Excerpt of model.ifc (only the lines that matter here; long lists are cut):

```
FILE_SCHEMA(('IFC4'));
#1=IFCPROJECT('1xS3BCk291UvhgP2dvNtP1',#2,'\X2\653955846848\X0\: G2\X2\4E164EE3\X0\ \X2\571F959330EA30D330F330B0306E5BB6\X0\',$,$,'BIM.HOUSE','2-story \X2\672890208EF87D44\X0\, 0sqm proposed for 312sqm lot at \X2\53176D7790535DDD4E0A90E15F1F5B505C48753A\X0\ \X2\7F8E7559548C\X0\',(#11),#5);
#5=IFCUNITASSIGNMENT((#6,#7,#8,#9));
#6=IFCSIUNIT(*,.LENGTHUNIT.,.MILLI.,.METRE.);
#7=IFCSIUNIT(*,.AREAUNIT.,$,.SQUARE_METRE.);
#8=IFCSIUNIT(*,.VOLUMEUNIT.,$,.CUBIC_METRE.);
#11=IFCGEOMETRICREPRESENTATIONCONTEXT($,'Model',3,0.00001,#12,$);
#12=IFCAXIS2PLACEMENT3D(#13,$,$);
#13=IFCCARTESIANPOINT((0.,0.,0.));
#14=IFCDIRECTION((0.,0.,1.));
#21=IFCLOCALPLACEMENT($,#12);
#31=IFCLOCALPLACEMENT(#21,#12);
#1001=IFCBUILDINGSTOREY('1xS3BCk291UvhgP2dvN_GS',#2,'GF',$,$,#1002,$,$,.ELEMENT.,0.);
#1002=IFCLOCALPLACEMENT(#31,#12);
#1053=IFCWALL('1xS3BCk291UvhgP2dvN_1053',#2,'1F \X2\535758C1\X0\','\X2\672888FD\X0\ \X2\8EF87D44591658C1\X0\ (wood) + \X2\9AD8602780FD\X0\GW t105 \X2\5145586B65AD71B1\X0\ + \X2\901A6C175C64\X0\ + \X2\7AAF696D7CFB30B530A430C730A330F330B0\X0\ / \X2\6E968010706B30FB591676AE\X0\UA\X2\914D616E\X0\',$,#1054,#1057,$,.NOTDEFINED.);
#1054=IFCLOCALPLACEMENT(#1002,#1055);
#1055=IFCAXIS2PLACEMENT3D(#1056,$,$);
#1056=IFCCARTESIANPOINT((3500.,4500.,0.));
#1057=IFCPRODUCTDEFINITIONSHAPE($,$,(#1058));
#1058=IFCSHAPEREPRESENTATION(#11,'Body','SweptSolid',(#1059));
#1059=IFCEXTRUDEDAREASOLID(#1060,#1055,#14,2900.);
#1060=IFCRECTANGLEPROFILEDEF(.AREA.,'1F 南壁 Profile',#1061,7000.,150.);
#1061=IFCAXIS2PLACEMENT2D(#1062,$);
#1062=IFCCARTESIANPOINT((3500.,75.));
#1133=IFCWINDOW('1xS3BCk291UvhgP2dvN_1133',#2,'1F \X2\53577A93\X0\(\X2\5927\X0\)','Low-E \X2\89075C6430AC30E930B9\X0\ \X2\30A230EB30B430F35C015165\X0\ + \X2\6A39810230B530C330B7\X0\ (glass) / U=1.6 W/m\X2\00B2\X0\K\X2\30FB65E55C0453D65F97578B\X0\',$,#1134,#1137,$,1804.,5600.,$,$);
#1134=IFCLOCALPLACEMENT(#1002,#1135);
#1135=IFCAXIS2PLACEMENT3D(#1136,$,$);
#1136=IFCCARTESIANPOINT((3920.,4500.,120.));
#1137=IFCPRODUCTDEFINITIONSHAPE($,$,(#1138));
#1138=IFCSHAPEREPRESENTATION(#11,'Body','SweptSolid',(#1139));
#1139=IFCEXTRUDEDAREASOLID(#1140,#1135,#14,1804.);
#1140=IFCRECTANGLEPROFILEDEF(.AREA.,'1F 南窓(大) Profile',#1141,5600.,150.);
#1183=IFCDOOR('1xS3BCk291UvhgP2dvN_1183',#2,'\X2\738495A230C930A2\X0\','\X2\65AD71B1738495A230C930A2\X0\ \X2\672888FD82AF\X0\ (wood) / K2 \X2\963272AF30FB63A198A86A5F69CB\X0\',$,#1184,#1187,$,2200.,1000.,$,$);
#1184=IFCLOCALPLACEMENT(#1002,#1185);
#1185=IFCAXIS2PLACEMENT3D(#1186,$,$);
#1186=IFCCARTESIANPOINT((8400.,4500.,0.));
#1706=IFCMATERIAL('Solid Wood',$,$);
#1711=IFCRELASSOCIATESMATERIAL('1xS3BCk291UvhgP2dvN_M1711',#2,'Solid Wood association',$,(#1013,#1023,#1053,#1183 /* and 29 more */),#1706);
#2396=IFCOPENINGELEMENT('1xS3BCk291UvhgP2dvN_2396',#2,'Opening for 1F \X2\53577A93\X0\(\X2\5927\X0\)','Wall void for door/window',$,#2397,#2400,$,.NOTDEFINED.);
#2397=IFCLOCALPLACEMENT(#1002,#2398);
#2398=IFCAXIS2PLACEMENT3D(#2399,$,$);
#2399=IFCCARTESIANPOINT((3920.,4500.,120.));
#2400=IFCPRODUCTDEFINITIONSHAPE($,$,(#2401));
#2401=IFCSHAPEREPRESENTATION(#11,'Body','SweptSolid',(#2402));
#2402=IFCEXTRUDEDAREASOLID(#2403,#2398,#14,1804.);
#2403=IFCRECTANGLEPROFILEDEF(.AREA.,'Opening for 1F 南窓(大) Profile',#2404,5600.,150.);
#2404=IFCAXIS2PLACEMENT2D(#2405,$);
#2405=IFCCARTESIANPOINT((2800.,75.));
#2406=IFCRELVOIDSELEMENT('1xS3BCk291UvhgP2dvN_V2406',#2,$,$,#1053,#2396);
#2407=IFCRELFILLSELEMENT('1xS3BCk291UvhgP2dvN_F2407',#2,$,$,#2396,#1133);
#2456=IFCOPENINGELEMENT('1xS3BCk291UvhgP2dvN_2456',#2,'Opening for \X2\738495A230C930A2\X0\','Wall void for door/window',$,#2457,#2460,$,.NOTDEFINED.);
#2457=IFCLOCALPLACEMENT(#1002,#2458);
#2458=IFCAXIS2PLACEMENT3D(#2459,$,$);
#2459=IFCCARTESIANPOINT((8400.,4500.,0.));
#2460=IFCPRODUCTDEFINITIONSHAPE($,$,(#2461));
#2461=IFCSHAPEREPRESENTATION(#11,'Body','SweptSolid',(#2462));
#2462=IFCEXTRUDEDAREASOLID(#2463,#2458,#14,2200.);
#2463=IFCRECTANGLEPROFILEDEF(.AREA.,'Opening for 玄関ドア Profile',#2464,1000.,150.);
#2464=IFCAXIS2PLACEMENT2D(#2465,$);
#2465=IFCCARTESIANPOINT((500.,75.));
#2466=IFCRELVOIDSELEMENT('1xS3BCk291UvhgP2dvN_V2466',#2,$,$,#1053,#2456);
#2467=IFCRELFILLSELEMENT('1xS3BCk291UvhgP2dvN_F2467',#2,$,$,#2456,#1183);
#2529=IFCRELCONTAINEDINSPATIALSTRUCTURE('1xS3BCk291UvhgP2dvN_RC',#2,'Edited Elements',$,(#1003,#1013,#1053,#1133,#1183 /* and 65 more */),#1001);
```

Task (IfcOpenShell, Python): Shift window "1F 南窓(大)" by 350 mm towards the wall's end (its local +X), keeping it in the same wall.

```python
import ifcopenshell
import ifcopenshell.api.geometry
import ifcopenshell.util.placement
import ifcopenshell.util.unit

model = ifcopenshell.open("model.ifc")
unit_scale = ifcopenshell.util.unit.calculate_unit_scale(model)

window = model.by_guid("1xS3BCk291UvhgP2dvN_1133")
opening = window.FillsVoids[0].RelatingOpeningElement
wall = opening.VoidsElements[0].RelatingBuildingElement

wall_matrix = ifcopenshell.util.placement.get_local_placement(wall.ObjectPlacement)
shift = wall_matrix[:3, 0] * 0.35 / unit_scale
before = ifcopenshell.util.placement.get_local_placement(window.ObjectPlacement)[:3, 3].copy()

# The window is not placed relative to its opening, so move both.
for product in (opening, window):
    matrix = ifcopenshell.util.placement.get_local_placement(product.ObjectPlacement)
    matrix[:3, 3] += shift
    ifcopenshell.api.geometry.edit_object_placement(model, product=product, matrix=matrix, is_si=False)

after = ifcopenshell.util.placement.get_local_placement(window.ObjectPlacement)[:3, 3]
print("window moved by", (after - before).round(3) + 0.0)

model.write("model_edited.ifc")
```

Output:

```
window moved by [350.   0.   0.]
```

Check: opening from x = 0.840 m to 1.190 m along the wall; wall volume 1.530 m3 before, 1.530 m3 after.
